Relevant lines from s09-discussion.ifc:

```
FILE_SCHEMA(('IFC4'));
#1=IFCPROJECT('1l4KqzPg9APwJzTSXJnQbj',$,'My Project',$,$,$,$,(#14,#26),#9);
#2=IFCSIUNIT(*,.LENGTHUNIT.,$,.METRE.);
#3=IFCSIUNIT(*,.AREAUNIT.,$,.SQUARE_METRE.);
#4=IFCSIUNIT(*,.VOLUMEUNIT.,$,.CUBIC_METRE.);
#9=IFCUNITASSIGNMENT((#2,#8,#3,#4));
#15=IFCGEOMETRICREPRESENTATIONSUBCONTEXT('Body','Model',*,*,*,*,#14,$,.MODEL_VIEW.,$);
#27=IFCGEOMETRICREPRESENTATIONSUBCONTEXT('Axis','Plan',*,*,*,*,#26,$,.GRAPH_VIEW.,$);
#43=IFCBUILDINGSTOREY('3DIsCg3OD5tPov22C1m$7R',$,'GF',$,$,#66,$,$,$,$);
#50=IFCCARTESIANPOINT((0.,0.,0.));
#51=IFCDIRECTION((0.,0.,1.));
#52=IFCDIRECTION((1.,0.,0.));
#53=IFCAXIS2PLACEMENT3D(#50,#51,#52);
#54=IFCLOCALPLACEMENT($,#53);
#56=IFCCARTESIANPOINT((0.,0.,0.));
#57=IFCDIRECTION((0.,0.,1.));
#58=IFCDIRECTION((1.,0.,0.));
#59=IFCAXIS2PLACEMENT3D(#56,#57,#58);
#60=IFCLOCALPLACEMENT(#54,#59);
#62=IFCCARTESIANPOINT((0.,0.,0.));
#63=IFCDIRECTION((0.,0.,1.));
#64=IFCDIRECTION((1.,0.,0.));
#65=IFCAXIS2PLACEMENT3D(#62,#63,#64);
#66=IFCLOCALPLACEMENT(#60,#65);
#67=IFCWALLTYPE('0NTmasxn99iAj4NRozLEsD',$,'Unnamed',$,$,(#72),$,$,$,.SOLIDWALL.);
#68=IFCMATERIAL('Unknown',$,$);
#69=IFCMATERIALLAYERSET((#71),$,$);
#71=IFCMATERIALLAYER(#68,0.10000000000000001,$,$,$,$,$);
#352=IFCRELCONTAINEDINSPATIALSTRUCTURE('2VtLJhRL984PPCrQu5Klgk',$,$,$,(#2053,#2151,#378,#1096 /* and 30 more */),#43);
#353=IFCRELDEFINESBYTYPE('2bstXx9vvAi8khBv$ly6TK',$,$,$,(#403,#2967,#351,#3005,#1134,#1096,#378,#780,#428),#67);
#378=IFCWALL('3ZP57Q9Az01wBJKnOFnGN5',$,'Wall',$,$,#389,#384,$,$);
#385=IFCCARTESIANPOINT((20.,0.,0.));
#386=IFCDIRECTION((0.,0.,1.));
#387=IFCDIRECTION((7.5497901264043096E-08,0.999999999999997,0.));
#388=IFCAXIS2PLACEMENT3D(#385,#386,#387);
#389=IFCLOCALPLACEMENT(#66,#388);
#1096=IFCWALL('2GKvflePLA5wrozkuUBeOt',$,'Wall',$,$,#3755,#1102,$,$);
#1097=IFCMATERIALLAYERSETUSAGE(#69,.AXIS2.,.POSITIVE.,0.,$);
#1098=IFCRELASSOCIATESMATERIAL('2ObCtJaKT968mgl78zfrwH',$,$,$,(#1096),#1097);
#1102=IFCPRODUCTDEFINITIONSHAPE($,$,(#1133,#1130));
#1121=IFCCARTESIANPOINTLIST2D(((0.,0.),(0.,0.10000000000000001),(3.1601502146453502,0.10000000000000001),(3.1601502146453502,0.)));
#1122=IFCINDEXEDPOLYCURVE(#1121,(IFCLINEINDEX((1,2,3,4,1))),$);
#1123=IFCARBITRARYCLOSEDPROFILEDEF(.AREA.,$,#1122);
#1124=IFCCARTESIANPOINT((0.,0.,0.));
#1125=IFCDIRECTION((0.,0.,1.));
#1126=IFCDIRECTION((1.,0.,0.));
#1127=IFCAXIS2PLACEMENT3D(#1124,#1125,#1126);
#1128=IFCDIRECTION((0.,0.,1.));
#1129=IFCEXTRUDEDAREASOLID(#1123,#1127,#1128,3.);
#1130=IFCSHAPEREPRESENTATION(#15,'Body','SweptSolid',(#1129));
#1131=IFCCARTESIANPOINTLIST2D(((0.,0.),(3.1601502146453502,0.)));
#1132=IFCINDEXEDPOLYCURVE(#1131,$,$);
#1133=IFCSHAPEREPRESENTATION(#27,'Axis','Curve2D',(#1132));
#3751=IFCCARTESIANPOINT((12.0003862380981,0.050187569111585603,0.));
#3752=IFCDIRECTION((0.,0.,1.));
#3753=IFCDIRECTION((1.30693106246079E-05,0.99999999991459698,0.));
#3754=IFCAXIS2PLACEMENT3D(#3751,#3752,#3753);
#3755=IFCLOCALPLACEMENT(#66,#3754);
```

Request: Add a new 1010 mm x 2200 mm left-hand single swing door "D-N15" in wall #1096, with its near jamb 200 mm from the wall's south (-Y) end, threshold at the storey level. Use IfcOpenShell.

```python
import numpy as np
import ifcopenshell
import ifcopenshell.api.feature
import ifcopenshell.api.geometry
import ifcopenshell.api.root
import ifcopenshell.api.spatial
import ifcopenshell.geom
import ifcopenshell.util.element
import ifcopenshell.util.placement
import ifcopenshell.util.representation
import ifcopenshell.util.shape
import ifcopenshell.util.unit

model = ifcopenshell.open("s09-discussion.ifc")
unit_scale = ifcopenshell.util.unit.calculate_unit_scale(model)
settings = ifcopenshell.geom.settings()


def volume(element):
    """Net volume in cubic metres, openings subtracted."""
    shape = ifcopenshell.geom.create_shape(settings, element)
    return ifcopenshell.util.shape.get_volume(shape.geometry)


wall = model.by_guid("2GKvflePLA5wrozkuUBeOt")
storey = ifcopenshell.util.element.get_container(wall, ifc_class="IfcBuildingStorey")
context = ifcopenshell.util.representation.get_context(model, "Model", "Body", "MODEL_VIEW")
before = volume(wall)

width, height, from_end, sill = 1.01, 2.2, 0.2, 0.0  # metres

# The wall runs along its own X axis, and the end named is its -X end.
wall_shape = ifcopenshell.geom.create_shape(settings, wall)
x, y, z = ifcopenshell.util.shape.get_vertices(wall_shape.geometry).T
start = x.min() + from_end
face, thickness = float(y.min()), float(y.max() - y.min())
wall_matrix = ifcopenshell.util.placement.get_local_placement(wall.ObjectPlacement)
level = ifcopenshell.util.placement.get_local_placement(storey.ObjectPlacement)[2, 3]


def in_wall(x, y):
    """Placement at x, y metres in the wall's axes, at sill height."""
    matrix = wall_matrix.copy()
    matrix[:, 3] = wall_matrix @ np.array([x / unit_scale, y / unit_scale, 0.0, 1.0])
    matrix[2, 3] = level + sill / unit_scale
    return matrix


# Opening: a box that overshoots both wall faces by 50 mm.
opening = ifcopenshell.api.root.create_entity(model, ifc_class="IfcOpeningElement", predefined_type="OPENING")
box = ifcopenshell.api.geometry.add_wall_representation(
    model, context=context, length=width, height=height, thickness=thickness + 0.1
)
ifcopenshell.api.geometry.assign_representation(model, product=opening, representation=box)
ifcopenshell.api.geometry.edit_object_placement(model, product=opening, matrix=in_wall(start, face - 0.05), is_si=False)
ifcopenshell.api.feature.add_feature(model, feature=opening, element=wall)

door = ifcopenshell.api.root.create_entity(model, ifc_class="IfcDoor", name="D-N15", predefined_type="DOOR")
door.OverallWidth, door.OverallHeight = width / unit_scale, height / unit_scale
door.OperationType = "SINGLE_SWING_LEFT"
body = ifcopenshell.api.geometry.add_door_representation(
    model,
    context=context,
    overall_width=door.OverallWidth,
    overall_height=door.OverallHeight,
    operation_type="SINGLE_SWING_LEFT",
    lining_properties={"LiningDepth": thickness / unit_scale, "ThresholdDepth": thickness / unit_scale},
)
ifcopenshell.api.geometry.assign_representation(model, product=door, representation=body)
ifcopenshell.api.spatial.assign_container(model, products=[door], relating_structure=storey)
ifcopenshell.api.feature.add_filling(model, opening=opening, element=door)

# The lining spans the wall, so the door starts at the wall face.
ifcopenshell.api.geometry.edit_object_placement(model, product=door, matrix=in_wall(start, face), is_si=False)

after = volume(wall)

print(f"wall volume {before:.3f} -> {after:.3f} m3")

model.write("s09-discussion-out.ifc")
```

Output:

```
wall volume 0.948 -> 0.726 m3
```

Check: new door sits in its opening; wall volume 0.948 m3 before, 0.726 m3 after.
